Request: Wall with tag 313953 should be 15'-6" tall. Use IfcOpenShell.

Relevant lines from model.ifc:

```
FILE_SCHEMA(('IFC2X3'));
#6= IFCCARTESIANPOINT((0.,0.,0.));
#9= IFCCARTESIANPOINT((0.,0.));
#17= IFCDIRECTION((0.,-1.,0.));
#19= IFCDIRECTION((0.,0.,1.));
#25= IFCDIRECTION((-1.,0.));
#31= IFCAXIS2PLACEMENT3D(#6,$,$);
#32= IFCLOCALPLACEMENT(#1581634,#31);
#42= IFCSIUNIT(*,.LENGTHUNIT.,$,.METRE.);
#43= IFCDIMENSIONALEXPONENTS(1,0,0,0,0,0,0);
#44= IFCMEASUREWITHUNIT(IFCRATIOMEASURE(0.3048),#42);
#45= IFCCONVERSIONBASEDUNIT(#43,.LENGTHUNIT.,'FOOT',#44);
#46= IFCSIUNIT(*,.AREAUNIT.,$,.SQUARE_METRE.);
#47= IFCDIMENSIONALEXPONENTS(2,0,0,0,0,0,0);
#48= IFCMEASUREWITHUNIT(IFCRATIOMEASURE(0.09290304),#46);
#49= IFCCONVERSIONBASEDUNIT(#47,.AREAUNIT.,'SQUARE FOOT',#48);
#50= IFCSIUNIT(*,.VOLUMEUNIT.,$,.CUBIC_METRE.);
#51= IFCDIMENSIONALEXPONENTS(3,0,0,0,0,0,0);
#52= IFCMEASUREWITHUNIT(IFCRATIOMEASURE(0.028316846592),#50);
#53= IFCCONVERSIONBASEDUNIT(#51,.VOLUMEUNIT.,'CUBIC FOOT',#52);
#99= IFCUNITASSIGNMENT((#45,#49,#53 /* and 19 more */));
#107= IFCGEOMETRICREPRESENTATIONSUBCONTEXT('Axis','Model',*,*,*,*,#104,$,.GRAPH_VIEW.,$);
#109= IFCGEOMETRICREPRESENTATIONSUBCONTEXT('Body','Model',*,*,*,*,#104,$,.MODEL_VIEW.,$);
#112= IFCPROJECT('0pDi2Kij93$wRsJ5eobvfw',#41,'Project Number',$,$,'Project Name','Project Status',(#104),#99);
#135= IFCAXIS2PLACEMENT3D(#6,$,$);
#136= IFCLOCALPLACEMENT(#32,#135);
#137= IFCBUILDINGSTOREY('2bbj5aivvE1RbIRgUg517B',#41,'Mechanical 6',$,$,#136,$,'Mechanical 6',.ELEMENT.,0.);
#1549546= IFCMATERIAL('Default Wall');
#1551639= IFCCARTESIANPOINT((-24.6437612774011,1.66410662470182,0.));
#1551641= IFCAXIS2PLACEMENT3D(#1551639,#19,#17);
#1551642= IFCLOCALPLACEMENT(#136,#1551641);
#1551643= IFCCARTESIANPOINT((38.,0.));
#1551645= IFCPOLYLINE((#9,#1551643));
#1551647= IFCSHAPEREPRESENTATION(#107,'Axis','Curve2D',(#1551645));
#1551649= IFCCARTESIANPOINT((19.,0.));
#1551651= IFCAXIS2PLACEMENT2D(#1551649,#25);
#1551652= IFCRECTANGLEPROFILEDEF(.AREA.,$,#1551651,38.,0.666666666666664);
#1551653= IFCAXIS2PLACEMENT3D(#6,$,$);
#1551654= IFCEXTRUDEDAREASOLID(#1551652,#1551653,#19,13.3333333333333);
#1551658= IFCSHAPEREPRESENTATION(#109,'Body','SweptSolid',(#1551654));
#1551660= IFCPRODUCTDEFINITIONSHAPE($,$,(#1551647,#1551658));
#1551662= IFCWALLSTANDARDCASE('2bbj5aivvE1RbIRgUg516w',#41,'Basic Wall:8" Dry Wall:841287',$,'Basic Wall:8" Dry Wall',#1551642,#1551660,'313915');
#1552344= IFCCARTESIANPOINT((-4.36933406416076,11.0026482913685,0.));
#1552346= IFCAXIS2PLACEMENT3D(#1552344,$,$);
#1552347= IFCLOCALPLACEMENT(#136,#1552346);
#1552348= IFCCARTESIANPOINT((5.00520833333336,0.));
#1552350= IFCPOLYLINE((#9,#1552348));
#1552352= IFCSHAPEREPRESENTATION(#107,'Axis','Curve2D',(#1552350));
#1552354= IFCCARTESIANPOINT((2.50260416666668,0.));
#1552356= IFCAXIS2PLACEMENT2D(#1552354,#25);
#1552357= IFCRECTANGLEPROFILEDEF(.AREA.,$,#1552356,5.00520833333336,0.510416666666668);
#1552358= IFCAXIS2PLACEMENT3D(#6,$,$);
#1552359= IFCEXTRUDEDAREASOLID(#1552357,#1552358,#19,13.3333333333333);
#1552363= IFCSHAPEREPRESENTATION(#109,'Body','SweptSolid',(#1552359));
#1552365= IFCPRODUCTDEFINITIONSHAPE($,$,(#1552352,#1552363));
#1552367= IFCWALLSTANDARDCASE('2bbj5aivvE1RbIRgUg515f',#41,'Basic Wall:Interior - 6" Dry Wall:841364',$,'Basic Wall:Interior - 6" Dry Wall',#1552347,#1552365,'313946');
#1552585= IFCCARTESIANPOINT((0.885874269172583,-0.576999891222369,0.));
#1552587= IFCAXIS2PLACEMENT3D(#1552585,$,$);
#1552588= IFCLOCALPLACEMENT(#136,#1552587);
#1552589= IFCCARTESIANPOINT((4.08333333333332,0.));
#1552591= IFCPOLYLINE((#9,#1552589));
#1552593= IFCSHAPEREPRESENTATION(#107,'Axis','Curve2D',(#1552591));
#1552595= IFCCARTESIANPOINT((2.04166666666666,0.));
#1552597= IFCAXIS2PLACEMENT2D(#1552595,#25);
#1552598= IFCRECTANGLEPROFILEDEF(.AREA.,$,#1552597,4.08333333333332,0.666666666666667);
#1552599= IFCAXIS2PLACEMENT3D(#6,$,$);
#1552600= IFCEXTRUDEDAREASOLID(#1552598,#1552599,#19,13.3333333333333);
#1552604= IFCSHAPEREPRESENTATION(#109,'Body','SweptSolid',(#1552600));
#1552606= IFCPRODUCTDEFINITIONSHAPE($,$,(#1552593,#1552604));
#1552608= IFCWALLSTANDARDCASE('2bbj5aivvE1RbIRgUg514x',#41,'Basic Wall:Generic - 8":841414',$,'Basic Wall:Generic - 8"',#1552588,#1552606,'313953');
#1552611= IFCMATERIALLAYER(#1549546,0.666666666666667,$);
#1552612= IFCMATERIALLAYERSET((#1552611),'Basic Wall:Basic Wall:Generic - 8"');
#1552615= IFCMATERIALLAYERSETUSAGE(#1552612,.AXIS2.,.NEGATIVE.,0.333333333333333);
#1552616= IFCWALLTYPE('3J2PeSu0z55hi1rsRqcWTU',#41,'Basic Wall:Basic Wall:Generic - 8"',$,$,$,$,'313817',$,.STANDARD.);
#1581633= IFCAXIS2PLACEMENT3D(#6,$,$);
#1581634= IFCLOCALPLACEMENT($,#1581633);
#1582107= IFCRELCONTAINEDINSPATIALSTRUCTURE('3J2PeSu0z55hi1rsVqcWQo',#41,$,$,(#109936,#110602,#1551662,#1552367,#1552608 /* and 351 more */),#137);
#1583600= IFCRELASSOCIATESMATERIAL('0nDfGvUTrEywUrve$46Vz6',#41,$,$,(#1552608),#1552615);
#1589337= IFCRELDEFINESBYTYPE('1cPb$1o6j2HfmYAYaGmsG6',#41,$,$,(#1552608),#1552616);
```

```python
import ifcopenshell
import ifcopenshell.geom
import ifcopenshell.util.representation
import ifcopenshell.util.shape
import ifcopenshell.util.unit

model = ifcopenshell.open("model.ifc")
unit_scale = ifcopenshell.util.unit.calculate_unit_scale(model)
settings = ifcopenshell.geom.settings()


def volume(element):
    """Net volume in cubic metres, openings subtracted."""
    shape = ifcopenshell.geom.create_shape(settings, element)
    return ifcopenshell.util.shape.get_volume(shape.geometry)


wall = model.by_id(1552608)
before = volume(wall)

body = ifcopenshell.util.representation.get_representation(wall, "Model", "Body")
solid = body.Items[0]
old_height = solid.Depth
solid.Depth = 186 * 0.0254 / unit_scale
after = volume(wall)

print(f"height {old_height:g} -> {solid.Depth:g}, volume {before:.3f} -> {after:.3f} m3")

model.write("model_rev.ifc")
```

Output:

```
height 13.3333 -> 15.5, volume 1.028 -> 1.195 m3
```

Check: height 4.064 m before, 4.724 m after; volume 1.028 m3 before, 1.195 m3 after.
